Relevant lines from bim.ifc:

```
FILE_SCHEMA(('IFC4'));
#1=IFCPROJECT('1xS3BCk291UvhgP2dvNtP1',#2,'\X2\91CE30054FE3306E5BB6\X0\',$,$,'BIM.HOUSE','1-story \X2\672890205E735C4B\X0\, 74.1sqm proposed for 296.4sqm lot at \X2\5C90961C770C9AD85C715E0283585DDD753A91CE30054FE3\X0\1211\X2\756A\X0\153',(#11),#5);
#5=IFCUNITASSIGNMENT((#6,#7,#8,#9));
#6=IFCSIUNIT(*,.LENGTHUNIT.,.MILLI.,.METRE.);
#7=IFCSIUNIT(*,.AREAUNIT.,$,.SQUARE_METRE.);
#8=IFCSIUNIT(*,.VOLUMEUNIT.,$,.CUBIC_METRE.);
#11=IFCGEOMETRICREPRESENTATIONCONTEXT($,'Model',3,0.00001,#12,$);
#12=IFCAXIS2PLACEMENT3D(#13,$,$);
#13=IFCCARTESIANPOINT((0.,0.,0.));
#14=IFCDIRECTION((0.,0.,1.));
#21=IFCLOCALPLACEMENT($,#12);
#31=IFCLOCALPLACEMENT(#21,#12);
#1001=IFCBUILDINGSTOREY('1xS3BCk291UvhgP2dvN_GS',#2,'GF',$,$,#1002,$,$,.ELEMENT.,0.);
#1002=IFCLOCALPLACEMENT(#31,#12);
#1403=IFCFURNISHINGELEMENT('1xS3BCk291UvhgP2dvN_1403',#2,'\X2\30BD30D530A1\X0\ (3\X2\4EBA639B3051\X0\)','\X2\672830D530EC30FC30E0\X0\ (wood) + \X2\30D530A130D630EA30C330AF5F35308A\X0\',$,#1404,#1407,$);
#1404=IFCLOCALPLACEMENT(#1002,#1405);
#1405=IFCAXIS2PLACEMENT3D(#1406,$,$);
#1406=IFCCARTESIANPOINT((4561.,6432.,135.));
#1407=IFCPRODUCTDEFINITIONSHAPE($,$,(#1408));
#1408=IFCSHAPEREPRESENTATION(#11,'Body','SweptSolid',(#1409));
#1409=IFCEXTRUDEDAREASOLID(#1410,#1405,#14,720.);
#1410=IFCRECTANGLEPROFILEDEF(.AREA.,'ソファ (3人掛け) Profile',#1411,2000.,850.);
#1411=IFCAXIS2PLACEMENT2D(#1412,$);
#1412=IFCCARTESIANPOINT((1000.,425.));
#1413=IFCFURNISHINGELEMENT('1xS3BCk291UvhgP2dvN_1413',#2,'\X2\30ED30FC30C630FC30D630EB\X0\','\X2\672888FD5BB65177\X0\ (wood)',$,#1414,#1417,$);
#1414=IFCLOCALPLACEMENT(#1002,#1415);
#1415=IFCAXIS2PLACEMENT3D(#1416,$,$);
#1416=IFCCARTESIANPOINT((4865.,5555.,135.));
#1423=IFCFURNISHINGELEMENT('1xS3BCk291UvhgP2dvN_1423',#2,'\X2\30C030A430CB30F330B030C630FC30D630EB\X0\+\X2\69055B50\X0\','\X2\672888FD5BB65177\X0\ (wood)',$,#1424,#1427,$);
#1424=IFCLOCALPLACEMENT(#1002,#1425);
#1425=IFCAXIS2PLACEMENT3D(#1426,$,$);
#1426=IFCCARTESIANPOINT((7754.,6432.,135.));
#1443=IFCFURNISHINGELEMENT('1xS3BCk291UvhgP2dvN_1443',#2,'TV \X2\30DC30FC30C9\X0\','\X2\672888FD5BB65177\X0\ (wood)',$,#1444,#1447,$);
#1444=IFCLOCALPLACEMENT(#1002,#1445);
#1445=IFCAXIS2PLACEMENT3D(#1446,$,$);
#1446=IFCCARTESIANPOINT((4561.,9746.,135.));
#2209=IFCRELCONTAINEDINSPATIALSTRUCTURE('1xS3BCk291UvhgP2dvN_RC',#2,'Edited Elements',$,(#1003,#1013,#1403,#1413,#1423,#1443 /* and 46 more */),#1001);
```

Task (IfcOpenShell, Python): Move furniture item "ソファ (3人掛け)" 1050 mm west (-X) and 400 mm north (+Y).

```python
import ifcopenshell
import ifcopenshell.api.geometry
import ifcopenshell.util.placement
import ifcopenshell.util.unit

model = ifcopenshell.open("bim.ifc")
unit_scale = ifcopenshell.util.unit.calculate_unit_scale(model)

item = model.by_guid("1xS3BCk291UvhgP2dvN_1403")
matrix = ifcopenshell.util.placement.get_local_placement(item.ObjectPlacement)
matrix[0, 3] -= 1.05 / unit_scale
matrix[1, 3] += 0.4 / unit_scale
ifcopenshell.api.geometry.edit_object_placement(model, product=item, matrix=matrix, is_si=False)

print(ifcopenshell.util.placement.get_local_placement(item.ObjectPlacement).round(3) + 0.0)

model.write("bim_edited.ifc")
```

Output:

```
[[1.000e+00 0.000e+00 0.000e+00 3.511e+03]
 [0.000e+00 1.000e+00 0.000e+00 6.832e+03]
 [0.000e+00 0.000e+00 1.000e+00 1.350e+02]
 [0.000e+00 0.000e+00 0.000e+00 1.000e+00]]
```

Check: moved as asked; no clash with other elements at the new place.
